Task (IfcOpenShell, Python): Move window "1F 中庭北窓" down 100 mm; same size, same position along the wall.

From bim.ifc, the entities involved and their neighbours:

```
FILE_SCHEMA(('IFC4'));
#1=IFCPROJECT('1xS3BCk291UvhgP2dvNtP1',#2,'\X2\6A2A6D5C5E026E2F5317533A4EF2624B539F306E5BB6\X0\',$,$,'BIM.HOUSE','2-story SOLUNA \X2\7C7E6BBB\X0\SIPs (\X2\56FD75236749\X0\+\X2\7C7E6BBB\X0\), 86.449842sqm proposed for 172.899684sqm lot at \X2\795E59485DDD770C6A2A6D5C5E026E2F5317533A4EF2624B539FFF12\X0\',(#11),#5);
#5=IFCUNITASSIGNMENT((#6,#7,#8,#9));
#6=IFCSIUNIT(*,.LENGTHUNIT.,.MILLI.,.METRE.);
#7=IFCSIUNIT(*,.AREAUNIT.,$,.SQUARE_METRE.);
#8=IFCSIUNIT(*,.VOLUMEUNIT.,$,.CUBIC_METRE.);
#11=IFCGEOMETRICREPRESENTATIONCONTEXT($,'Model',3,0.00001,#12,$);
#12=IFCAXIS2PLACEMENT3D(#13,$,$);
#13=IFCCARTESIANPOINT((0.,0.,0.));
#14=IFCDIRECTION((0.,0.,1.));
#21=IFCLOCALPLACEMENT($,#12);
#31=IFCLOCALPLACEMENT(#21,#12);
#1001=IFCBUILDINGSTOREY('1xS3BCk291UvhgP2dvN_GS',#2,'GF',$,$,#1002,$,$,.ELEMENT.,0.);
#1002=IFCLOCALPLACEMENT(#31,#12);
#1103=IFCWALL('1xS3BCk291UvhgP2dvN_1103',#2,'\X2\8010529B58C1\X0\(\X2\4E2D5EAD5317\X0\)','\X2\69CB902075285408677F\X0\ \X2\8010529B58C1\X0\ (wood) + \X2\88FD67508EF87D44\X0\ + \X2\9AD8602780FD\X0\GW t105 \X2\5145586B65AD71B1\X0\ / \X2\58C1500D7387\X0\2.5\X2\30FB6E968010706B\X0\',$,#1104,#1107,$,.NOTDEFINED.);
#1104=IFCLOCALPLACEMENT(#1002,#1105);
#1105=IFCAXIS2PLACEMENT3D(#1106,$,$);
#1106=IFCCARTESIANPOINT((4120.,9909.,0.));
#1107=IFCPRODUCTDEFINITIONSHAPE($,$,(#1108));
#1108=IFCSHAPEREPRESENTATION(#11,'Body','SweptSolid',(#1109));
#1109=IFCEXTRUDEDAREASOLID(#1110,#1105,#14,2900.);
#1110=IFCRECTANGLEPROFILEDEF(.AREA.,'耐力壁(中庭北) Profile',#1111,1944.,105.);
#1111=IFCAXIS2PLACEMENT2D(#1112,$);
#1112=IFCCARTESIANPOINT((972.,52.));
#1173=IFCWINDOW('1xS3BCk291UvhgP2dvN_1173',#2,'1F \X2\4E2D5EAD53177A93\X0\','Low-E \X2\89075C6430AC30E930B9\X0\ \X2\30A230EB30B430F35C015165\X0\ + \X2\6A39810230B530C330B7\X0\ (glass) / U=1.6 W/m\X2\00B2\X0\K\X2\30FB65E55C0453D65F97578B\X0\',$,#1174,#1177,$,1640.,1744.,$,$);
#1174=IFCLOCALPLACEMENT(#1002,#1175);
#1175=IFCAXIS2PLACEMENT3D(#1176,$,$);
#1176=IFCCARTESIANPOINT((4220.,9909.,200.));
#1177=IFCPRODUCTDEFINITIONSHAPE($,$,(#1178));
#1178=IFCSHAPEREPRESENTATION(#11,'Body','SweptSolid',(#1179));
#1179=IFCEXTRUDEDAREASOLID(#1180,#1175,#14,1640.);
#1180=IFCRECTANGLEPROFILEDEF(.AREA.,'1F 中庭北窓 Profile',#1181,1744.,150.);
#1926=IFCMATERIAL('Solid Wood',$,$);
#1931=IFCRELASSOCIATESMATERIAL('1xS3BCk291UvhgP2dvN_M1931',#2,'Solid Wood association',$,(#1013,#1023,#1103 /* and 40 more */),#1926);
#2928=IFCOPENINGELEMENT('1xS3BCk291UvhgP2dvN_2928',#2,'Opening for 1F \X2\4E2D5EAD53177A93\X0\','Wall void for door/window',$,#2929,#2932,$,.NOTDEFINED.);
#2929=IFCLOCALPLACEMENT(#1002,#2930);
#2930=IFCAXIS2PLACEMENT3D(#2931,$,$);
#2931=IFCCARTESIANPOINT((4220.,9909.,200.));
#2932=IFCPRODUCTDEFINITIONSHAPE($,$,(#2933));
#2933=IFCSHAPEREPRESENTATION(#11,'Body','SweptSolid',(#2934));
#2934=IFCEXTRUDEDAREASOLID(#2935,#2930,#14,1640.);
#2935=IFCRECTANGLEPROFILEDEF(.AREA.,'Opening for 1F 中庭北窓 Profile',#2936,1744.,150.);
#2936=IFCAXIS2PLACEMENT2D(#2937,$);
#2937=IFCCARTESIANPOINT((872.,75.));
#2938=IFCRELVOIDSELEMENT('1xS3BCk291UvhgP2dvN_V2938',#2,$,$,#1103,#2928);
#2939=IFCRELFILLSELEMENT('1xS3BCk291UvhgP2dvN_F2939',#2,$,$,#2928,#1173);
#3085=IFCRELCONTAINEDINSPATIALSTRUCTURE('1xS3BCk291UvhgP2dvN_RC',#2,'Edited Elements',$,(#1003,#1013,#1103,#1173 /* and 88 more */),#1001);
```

```python
import numpy as np
import ifcopenshell
import ifcopenshell.api.geometry
import ifcopenshell.util.placement
import ifcopenshell.util.unit

model = ifcopenshell.open("bim.ifc")
unit_scale = ifcopenshell.util.unit.calculate_unit_scale(model)

window = model.by_guid("1xS3BCk291UvhgP2dvN_1173")
opening = window.FillsVoids[0].RelatingOpeningElement
dz = -0.1 / unit_scale

shift = np.array([0.0, 0.0, dz])
# The window is not placed relative to its opening, so move both.
for product in (opening, window):
    matrix = ifcopenshell.util.placement.get_local_placement(product.ObjectPlacement)
    matrix[:3, 3] += shift
    ifcopenshell.api.geometry.edit_object_placement(model, product=product, matrix=matrix, is_si=False)

print(f"moved by {dz * unit_scale:+.3f} m")

model.write("bim_v2.ifc")
```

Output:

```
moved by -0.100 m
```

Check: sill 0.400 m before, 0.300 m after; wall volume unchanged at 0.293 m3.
